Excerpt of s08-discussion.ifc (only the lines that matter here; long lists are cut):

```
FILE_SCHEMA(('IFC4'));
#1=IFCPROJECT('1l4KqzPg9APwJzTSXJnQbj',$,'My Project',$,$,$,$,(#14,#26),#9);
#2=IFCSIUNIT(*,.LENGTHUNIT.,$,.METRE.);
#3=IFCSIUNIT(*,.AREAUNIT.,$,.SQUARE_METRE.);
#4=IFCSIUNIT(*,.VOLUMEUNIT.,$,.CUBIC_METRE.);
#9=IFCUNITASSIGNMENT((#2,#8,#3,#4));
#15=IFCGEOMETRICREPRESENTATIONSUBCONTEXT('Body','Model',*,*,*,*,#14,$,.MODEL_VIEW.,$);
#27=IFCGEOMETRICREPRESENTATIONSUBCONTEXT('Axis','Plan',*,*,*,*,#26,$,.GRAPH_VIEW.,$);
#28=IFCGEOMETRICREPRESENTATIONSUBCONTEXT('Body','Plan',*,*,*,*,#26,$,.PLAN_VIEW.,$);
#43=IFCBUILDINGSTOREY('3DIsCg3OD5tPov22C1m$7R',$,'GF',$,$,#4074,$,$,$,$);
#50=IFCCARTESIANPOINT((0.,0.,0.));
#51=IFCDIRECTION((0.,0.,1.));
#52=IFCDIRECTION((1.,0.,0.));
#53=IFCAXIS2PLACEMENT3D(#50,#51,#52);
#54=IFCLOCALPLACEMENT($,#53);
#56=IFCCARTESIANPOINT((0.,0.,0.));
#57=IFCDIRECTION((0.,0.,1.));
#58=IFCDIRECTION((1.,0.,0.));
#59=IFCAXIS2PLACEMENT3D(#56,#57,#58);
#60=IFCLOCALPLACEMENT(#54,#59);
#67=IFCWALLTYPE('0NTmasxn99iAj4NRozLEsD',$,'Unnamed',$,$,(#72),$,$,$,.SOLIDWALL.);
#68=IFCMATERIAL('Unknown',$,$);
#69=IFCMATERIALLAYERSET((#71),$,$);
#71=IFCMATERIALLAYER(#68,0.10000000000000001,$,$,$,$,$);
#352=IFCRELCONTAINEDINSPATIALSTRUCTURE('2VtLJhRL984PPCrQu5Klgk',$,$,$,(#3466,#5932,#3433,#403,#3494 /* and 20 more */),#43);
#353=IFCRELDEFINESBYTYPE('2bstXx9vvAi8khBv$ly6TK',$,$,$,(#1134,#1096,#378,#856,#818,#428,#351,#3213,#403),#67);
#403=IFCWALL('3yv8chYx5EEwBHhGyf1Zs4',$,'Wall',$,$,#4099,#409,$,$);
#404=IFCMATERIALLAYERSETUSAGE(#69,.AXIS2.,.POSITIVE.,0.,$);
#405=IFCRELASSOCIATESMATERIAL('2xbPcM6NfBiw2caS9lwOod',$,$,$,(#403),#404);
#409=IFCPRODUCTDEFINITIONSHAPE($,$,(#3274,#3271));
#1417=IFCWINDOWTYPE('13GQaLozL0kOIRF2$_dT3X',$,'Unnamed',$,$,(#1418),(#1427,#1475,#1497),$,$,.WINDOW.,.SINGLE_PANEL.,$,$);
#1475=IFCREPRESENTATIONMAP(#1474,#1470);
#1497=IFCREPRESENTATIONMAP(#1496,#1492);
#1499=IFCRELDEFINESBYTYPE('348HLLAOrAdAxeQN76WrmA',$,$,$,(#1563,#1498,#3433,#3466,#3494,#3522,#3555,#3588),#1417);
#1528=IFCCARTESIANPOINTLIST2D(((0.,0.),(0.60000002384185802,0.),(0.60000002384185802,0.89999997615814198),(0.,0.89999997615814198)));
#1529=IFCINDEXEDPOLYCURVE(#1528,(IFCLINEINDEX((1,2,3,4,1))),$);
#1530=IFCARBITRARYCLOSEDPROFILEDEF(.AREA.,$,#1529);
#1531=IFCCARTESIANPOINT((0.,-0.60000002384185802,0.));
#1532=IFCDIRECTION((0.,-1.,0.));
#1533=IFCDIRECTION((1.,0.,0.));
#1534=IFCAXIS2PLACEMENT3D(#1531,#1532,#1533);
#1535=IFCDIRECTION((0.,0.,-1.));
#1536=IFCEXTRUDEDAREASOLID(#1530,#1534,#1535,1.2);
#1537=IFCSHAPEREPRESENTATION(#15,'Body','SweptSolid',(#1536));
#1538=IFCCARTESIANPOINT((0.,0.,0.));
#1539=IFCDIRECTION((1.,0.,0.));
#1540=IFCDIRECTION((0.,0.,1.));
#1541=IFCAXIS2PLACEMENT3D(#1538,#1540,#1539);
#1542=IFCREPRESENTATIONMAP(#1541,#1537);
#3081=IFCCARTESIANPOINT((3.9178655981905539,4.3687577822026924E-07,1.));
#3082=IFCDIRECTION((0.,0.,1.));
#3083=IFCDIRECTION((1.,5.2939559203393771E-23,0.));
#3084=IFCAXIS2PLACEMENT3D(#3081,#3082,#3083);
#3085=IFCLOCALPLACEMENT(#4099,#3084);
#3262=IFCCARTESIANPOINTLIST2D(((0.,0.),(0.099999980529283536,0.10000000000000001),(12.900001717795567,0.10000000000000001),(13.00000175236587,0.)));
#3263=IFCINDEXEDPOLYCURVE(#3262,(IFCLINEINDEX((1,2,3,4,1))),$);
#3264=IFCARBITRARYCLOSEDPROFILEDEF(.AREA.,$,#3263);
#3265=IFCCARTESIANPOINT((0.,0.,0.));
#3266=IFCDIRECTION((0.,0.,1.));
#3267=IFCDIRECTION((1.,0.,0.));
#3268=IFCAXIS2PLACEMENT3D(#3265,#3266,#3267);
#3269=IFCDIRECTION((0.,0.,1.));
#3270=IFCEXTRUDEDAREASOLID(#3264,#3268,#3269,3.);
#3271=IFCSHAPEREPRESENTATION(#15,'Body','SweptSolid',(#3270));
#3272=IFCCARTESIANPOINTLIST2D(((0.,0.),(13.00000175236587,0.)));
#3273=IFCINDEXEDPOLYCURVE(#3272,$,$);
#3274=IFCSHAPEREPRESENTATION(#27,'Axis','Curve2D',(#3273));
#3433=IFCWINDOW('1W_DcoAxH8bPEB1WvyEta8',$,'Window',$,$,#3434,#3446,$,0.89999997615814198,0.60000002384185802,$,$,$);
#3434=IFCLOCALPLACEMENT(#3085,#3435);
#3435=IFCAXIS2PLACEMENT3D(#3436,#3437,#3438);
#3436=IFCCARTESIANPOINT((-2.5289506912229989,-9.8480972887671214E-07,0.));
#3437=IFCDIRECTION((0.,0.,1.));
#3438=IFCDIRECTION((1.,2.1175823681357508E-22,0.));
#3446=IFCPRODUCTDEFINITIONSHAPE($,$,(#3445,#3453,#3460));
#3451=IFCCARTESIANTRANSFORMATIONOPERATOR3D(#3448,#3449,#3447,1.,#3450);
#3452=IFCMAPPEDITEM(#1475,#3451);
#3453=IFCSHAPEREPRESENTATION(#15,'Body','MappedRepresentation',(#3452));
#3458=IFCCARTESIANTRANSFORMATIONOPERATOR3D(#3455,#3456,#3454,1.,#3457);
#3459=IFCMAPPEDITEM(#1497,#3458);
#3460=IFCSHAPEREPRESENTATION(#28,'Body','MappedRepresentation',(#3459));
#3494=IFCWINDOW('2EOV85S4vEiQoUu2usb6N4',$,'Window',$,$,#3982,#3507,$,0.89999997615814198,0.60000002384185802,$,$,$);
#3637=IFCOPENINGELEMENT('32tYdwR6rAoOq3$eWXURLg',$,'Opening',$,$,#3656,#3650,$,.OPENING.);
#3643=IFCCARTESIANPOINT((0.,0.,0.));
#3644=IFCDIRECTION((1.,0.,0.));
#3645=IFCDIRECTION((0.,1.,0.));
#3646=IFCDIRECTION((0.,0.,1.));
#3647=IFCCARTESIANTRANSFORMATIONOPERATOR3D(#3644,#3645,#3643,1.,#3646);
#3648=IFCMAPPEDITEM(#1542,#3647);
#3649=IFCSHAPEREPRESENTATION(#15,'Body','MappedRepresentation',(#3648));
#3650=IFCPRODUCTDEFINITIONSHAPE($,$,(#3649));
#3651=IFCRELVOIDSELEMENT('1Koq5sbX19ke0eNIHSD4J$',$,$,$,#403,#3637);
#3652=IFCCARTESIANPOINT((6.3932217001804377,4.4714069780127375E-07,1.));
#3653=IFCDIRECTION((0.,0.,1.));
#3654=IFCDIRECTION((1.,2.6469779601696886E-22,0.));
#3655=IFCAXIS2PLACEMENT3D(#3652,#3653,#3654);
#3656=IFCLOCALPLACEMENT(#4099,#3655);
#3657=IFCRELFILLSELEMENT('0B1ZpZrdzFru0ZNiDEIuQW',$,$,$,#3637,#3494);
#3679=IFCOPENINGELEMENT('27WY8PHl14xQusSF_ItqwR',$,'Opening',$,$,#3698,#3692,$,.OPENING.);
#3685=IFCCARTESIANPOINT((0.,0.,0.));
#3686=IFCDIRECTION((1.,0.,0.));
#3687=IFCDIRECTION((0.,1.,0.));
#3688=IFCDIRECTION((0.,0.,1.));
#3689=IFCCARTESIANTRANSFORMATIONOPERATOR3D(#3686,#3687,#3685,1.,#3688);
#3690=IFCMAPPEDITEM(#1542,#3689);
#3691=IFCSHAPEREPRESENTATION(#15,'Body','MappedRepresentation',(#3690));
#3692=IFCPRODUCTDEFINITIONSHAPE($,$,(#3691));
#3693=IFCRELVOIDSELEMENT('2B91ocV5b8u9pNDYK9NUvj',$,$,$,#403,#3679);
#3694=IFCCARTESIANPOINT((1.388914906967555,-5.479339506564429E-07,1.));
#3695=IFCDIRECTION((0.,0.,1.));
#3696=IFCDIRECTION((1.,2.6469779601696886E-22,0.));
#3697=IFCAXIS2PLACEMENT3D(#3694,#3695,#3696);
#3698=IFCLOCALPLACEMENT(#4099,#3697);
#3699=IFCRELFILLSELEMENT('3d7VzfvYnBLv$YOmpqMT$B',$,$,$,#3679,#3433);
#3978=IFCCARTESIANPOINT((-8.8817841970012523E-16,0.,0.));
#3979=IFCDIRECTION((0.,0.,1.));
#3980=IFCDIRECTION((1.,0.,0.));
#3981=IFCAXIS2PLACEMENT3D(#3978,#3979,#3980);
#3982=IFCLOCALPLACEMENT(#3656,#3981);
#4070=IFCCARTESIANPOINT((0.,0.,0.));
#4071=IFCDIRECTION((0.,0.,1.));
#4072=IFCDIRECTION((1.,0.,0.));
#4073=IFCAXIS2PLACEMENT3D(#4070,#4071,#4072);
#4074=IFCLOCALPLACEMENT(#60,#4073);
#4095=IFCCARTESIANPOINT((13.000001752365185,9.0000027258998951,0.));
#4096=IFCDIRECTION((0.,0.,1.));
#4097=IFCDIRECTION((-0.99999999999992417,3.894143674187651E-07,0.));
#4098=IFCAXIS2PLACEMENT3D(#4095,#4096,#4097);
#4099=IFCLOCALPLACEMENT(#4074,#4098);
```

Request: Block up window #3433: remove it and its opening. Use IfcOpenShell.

```python
import ifcopenshell
import ifcopenshell.api.feature
import ifcopenshell.api.root
import ifcopenshell.geom
import ifcopenshell.util.shape

model = ifcopenshell.open("s08-discussion.ifc")
settings = ifcopenshell.geom.settings()


def volume(element):
    """Net volume in cubic metres, openings subtracted."""
    shape = ifcopenshell.geom.create_shape(settings, element)
    return ifcopenshell.util.shape.get_volume(shape.geometry)


window = model.by_guid("1W_DcoAxH8bPEB1WvyEta8")
opening = window.FillsVoids[0].RelatingOpeningElement
wall = opening.VoidsElements[0].RelatingBuildingElement
before = volume(wall)

ifcopenshell.api.root.remove_product(model, product=window)
ifcopenshell.api.feature.remove_feature(model, feature=opening)

after = volume(wall)

print(f"wall volume {before:.3f} -> {after:.3f} m3")

model.write("s08-discussion_updated.ifc")
```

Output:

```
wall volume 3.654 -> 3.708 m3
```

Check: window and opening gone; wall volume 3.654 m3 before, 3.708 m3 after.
